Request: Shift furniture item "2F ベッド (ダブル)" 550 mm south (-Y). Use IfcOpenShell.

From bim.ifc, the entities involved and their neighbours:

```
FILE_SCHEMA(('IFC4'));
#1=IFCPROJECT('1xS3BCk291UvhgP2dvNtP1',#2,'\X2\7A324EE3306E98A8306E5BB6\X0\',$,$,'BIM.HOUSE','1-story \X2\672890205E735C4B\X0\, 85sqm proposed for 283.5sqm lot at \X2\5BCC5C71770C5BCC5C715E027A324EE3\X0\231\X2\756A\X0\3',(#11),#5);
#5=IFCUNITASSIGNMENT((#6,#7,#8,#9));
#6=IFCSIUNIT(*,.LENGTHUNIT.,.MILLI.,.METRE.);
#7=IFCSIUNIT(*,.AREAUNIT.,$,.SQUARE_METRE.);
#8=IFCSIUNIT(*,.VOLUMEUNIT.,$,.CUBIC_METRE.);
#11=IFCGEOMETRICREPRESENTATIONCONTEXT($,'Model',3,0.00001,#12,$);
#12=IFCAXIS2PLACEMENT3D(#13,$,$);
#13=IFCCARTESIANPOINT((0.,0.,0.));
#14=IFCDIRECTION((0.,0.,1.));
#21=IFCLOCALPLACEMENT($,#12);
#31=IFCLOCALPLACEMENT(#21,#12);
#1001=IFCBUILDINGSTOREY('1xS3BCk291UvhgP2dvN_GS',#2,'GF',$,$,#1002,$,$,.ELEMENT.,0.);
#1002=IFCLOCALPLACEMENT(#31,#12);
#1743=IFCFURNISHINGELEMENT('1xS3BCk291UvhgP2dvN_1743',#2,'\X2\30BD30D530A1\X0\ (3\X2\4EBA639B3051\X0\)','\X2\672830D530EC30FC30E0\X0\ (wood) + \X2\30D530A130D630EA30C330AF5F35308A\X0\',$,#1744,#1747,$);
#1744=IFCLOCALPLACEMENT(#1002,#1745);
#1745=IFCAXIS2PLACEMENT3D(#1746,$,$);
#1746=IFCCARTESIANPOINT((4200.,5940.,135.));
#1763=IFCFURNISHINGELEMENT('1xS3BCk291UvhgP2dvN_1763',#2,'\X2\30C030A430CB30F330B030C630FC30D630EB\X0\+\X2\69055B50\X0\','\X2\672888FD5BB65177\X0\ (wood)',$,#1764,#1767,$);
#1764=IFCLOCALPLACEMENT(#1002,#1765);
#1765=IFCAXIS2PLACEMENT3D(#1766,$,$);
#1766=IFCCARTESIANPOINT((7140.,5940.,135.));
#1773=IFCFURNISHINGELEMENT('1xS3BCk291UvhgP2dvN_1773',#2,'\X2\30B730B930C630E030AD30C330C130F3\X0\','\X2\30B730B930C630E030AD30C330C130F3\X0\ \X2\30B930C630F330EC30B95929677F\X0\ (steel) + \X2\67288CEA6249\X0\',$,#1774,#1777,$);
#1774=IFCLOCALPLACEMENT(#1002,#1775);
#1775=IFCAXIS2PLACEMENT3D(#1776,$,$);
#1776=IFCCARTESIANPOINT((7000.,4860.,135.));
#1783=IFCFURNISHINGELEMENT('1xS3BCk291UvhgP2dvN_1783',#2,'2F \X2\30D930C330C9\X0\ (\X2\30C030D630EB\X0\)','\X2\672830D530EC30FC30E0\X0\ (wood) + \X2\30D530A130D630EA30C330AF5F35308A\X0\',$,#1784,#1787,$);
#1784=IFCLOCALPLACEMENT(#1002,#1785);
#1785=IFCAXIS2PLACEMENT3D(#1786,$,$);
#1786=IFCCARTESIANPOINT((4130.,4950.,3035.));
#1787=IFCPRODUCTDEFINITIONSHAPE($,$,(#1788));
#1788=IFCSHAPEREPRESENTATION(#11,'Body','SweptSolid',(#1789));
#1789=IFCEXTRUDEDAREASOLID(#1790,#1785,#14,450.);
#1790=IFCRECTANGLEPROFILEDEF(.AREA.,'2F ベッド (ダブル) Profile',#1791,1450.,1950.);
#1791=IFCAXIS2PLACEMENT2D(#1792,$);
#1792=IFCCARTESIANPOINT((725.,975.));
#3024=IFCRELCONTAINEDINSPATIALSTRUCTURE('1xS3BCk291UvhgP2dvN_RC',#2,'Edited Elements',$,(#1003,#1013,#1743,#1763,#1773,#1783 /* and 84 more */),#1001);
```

```python
import ifcopenshell
import ifcopenshell.api.geometry
import ifcopenshell.util.placement
import ifcopenshell.util.unit

model = ifcopenshell.open("bim.ifc")
unit_scale = ifcopenshell.util.unit.calculate_unit_scale(model)

item = model.by_id(1783)
matrix = ifcopenshell.util.placement.get_local_placement(item.ObjectPlacement)
matrix[1, 3] -= 0.55 / unit_scale
ifcopenshell.api.geometry.edit_object_placement(model, product=item, matrix=matrix, is_si=False)

print(ifcopenshell.util.placement.get_local_placement(item.ObjectPlacement).round(3) + 0.0)

model.write("bim_rev.ifc")
```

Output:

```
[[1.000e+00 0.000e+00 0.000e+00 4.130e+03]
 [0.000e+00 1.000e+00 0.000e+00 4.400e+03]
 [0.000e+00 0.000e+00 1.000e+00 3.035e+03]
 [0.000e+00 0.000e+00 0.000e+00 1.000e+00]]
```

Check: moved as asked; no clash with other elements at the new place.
